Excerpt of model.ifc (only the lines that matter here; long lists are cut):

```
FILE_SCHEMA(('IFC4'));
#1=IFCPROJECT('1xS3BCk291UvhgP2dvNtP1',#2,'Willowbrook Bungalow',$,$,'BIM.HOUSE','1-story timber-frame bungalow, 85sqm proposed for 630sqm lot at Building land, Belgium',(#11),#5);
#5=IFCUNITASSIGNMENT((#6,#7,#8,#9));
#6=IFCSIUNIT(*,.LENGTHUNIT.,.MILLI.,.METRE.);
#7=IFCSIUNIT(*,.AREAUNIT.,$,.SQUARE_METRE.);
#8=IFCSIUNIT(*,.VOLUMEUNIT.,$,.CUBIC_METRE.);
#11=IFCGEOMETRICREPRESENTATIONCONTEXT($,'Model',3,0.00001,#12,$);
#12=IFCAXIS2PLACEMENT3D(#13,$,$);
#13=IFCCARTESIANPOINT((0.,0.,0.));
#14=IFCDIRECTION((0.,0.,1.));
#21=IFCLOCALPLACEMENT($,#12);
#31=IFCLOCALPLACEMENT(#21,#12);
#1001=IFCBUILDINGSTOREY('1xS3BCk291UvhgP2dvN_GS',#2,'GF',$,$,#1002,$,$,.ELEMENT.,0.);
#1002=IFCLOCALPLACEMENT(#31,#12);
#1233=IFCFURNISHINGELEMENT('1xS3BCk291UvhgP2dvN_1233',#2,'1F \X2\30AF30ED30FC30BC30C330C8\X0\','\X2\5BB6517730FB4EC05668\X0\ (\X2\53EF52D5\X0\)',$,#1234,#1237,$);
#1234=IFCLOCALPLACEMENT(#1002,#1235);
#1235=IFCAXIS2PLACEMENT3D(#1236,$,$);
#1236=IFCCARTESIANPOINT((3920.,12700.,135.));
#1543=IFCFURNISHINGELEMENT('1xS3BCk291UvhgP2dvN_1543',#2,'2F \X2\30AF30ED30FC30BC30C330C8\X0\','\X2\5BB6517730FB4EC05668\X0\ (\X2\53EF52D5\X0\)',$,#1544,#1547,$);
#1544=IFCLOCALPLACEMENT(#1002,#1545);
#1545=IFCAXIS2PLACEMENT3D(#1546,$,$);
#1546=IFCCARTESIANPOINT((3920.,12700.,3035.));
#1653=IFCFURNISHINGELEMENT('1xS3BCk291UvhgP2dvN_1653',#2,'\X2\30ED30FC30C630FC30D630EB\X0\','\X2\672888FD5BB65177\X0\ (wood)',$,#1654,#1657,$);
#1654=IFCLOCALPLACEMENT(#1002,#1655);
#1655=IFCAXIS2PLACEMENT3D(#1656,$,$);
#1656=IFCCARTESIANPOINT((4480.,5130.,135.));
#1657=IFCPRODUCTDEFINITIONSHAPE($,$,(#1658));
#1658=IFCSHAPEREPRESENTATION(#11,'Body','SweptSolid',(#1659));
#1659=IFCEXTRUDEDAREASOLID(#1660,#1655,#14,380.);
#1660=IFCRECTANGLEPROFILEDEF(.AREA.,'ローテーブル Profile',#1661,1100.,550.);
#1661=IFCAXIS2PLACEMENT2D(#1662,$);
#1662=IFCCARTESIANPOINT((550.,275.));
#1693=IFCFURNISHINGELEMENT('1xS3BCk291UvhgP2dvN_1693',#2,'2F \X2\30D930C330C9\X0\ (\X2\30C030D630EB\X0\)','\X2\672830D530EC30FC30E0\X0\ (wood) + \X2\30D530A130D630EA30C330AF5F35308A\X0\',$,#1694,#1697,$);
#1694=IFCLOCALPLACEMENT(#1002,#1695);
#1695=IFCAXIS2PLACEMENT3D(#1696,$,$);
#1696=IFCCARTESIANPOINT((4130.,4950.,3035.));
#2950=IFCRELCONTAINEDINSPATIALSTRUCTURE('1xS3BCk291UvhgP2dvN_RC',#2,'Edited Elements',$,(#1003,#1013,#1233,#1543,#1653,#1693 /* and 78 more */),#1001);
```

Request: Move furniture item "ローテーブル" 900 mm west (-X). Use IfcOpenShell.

```python
import ifcopenshell
import ifcopenshell.api.geometry
import ifcopenshell.util.placement
import ifcopenshell.util.unit

model = ifcopenshell.open("model.ifc")
unit_scale = ifcopenshell.util.unit.calculate_unit_scale(model)

item = model.by_guid("1xS3BCk291UvhgP2dvN_1653")
matrix = ifcopenshell.util.placement.get_local_placement(item.ObjectPlacement)
matrix[0, 3] -= 0.9 / unit_scale
ifcopenshell.api.geometry.edit_object_placement(model, product=item, matrix=matrix, is_si=False)

print(ifcopenshell.util.placement.get_local_placement(item.ObjectPlacement).round(3) + 0.0)

model.write("model_updated.ifc")
```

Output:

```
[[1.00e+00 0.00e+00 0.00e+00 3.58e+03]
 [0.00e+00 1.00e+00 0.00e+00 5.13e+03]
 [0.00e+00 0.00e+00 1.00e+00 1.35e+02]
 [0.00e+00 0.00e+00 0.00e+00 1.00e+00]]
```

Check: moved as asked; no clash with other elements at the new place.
